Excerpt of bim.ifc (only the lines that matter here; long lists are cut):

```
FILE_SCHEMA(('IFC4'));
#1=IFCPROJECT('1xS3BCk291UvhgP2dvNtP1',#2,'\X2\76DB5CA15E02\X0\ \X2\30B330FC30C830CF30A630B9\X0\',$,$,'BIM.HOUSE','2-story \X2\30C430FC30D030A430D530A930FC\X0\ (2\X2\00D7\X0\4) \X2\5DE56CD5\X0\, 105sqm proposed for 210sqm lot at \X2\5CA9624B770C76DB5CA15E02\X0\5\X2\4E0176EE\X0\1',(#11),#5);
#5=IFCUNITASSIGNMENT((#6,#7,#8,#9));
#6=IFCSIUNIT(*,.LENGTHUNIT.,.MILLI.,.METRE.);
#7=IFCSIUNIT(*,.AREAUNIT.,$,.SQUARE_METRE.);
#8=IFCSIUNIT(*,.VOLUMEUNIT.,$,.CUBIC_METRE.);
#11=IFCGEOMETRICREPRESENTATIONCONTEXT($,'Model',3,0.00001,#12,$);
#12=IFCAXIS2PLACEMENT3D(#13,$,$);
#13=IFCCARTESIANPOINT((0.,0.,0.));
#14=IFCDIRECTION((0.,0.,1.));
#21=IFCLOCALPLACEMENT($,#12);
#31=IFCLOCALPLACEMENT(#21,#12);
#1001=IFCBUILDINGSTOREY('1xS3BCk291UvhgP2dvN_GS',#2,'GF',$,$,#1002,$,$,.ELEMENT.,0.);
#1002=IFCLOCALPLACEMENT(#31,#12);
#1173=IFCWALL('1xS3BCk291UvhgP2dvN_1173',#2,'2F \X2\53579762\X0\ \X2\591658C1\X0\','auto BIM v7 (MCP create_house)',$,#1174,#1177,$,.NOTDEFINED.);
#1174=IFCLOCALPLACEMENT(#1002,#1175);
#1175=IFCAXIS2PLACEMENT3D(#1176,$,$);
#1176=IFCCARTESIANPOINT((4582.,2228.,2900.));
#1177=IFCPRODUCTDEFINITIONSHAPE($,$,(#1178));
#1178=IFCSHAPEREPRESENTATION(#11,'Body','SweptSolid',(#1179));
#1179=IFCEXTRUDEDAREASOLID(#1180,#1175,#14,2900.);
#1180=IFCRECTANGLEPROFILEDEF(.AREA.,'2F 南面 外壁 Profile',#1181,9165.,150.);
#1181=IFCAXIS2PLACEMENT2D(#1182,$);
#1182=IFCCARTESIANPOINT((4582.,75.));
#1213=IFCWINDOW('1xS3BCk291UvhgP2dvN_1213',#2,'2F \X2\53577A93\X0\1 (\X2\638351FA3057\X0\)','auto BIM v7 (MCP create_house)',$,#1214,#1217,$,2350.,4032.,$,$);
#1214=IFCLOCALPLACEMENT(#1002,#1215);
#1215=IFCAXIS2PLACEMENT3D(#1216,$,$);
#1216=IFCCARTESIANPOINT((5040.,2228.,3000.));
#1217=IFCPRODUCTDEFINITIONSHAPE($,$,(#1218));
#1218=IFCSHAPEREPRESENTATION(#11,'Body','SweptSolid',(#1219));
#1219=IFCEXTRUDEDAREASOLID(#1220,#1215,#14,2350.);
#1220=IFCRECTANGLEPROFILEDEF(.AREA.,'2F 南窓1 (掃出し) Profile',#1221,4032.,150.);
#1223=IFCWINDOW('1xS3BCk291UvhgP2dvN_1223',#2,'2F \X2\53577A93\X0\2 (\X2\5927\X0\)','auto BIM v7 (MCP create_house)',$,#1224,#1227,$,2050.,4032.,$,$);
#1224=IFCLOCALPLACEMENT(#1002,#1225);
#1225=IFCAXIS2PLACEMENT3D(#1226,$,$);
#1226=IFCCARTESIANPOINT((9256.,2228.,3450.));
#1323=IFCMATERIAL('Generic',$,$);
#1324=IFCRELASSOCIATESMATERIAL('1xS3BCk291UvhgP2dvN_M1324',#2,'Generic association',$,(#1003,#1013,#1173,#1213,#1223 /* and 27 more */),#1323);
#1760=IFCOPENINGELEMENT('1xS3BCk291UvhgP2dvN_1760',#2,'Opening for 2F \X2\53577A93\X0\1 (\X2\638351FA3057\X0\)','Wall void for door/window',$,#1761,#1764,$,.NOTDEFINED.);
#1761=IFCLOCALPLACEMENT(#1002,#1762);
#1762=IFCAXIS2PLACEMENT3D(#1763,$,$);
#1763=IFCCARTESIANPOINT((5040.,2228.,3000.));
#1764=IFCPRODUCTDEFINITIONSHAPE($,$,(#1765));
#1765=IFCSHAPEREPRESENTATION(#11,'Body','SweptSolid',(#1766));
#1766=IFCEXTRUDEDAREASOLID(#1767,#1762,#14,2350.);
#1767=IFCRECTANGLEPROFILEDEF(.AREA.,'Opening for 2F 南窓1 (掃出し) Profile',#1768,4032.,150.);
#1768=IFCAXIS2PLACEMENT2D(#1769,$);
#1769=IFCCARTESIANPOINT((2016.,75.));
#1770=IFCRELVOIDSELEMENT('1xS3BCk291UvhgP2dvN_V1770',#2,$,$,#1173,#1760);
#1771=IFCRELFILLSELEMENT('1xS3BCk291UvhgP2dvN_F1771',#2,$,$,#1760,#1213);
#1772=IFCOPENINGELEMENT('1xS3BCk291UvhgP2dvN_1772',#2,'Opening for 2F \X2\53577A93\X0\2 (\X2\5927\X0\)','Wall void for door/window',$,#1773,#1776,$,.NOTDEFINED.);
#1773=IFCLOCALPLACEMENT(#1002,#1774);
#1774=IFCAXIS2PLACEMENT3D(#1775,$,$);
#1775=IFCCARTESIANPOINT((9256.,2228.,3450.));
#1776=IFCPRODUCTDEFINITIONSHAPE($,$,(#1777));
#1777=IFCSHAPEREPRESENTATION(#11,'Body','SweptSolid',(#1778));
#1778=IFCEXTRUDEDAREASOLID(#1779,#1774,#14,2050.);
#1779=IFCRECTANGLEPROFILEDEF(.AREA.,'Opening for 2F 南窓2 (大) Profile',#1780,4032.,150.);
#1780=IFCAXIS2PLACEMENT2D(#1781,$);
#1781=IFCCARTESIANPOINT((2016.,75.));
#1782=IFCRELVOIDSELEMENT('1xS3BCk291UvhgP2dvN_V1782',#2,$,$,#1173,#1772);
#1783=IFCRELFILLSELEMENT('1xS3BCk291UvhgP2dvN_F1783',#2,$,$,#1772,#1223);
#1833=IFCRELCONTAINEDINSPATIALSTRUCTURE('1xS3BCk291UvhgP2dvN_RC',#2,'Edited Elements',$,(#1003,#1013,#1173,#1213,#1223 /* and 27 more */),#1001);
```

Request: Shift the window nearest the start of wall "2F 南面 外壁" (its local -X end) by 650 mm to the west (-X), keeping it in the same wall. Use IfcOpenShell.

```python
import ifcopenshell
import ifcopenshell.api.geometry
import ifcopenshell.util.placement

model = ifcopenshell.open("bim.ifc")

window = model.by_id(1213)
opening = window.FillsVoids[0].RelatingOpeningElement
wall = opening.VoidsElements[0].RelatingBuildingElement

wall_matrix = ifcopenshell.util.placement.get_local_placement(wall.ObjectPlacement)
shift = wall_matrix[:3, 0] * -650.0
before = ifcopenshell.util.placement.get_local_placement(window.ObjectPlacement)[:3, 3].copy()

# The window is not placed relative to its opening, so move both.
for product in (opening, window):
    matrix = ifcopenshell.util.placement.get_local_placement(product.ObjectPlacement)
    matrix[:3, 3] += shift
    ifcopenshell.api.geometry.edit_object_placement(model, product=product, matrix=matrix, is_si=False)

after = ifcopenshell.util.placement.get_local_placement(window.ObjectPlacement)[:3, 3]
print("window moved by", (after - before).round(3) + 0.0)

model.write("bim_v2.ifc")
```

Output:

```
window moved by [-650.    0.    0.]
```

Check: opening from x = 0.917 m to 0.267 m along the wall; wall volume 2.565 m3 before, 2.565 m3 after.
